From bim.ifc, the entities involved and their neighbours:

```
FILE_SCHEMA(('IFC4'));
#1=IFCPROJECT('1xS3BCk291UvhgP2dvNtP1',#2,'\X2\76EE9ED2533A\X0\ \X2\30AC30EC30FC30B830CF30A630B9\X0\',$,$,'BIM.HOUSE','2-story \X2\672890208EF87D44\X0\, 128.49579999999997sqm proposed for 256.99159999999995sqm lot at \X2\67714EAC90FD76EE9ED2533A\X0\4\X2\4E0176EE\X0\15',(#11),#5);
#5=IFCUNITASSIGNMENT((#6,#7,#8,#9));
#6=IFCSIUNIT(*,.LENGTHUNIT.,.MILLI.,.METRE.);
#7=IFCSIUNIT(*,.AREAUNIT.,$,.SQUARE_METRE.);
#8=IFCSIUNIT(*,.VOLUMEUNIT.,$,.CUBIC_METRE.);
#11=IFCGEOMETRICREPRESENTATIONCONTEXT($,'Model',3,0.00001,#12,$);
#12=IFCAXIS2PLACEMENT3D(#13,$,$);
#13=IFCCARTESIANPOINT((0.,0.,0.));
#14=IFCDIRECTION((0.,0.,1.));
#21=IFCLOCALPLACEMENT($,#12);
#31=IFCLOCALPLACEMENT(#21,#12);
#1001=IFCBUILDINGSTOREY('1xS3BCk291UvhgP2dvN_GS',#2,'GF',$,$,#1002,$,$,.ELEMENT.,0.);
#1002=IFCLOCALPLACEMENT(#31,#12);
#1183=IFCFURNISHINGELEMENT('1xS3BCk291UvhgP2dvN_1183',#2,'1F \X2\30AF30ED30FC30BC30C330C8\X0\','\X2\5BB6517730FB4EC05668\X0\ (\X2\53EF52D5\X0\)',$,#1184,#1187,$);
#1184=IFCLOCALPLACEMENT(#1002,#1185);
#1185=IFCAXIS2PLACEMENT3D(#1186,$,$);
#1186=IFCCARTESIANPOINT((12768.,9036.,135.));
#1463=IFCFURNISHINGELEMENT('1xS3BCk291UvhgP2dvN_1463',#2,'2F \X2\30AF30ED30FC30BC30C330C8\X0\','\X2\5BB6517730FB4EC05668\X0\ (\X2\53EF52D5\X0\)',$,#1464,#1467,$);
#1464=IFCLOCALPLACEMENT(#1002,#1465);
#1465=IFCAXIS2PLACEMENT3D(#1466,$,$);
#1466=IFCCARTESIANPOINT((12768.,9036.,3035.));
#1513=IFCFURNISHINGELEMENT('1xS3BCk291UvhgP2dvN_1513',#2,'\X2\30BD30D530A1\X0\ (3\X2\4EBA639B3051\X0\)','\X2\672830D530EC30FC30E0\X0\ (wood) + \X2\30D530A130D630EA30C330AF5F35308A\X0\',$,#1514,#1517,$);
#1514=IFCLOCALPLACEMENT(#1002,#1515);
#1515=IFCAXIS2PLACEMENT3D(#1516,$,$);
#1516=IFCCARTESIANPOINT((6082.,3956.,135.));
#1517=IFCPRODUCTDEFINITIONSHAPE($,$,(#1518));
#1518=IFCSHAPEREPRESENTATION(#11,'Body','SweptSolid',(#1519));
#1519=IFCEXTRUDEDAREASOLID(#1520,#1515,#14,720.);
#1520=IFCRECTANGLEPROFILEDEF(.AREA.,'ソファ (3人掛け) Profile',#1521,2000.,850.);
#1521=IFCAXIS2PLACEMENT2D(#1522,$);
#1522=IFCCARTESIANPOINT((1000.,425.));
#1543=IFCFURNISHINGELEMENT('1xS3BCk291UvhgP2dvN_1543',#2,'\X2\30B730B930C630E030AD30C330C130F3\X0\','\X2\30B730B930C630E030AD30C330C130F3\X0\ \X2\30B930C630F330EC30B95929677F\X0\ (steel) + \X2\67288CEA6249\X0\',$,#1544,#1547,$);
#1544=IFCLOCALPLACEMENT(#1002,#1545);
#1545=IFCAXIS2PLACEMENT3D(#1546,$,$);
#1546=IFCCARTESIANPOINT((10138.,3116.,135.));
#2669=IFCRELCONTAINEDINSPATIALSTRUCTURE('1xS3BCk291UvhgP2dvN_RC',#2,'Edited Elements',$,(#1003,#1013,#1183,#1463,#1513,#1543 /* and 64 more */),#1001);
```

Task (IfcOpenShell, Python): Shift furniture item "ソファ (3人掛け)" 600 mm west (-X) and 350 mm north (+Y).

```python
import ifcopenshell
import ifcopenshell.api.geometry
import ifcopenshell.util.placement

model = ifcopenshell.open("bim.ifc")

item = model.by_id(1513)
matrix = ifcopenshell.util.placement.get_local_placement(item.ObjectPlacement)
matrix[0, 3] -= 600.0
matrix[1, 3] += 350.0
ifcopenshell.api.geometry.edit_object_placement(model, product=item, matrix=matrix, is_si=False)

print(ifcopenshell.util.placement.get_local_placement(item.ObjectPlacement).round(3) + 0.0)

model.write("bim-out.ifc")
```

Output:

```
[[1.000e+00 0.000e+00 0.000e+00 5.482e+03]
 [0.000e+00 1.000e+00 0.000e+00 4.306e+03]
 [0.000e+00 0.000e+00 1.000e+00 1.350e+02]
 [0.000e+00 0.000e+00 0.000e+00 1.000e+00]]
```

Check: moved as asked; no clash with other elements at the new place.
